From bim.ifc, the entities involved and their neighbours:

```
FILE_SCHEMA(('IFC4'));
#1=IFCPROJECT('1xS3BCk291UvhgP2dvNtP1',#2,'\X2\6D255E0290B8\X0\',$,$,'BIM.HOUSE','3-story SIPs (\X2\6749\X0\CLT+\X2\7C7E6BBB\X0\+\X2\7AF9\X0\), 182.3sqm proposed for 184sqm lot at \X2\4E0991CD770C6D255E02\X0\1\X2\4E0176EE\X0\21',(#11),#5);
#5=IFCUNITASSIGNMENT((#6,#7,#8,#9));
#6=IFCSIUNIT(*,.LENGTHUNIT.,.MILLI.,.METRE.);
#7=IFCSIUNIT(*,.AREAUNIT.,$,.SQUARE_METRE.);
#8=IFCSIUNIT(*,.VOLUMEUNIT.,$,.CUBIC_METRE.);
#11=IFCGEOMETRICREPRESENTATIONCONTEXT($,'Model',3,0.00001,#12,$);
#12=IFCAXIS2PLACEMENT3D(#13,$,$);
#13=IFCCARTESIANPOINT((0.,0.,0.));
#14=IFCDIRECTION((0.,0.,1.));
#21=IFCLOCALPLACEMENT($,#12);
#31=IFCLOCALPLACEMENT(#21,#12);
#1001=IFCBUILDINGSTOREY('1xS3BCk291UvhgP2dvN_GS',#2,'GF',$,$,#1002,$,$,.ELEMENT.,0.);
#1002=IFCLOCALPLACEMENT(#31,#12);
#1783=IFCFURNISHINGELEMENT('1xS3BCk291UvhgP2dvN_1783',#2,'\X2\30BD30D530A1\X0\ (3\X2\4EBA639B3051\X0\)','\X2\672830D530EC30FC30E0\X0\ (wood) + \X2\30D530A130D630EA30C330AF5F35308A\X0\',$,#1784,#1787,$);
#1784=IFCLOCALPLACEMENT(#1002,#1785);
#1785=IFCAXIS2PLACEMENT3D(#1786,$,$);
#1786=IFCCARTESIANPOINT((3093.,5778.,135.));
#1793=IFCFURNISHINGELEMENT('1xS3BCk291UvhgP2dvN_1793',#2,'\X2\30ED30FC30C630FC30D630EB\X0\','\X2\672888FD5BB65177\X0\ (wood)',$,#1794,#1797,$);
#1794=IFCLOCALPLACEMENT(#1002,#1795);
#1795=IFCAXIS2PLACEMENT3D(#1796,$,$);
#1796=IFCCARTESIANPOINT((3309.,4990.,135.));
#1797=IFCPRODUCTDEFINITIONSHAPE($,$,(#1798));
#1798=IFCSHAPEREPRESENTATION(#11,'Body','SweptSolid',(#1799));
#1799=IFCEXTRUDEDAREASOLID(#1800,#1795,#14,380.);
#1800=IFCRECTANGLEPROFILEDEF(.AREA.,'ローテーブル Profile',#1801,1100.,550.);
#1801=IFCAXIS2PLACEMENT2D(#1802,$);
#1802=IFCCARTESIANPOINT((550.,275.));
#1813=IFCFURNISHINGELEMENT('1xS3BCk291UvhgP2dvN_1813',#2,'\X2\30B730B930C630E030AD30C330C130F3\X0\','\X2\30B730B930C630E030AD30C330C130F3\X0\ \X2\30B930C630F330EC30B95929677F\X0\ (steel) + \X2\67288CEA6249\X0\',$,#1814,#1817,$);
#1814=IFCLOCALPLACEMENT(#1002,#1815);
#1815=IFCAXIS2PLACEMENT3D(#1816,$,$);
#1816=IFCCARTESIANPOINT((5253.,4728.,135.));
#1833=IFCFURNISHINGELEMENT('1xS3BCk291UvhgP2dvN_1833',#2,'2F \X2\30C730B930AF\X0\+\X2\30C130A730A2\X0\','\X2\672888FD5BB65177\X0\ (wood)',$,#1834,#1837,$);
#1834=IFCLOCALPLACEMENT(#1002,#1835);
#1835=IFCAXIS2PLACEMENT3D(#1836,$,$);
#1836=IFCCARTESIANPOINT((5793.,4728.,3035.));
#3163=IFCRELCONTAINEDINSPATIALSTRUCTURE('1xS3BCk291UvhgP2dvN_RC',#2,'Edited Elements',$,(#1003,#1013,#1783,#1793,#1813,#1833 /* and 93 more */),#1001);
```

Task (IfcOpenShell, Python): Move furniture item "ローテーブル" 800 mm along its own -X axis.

```python
import ifcopenshell
import ifcopenshell.api.geometry
import ifcopenshell.util.placement
import ifcopenshell.util.unit

model = ifcopenshell.open("bim.ifc")
unit_scale = ifcopenshell.util.unit.calculate_unit_scale(model)

item = model.by_guid("1xS3BCk291UvhgP2dvN_1793")
matrix = ifcopenshell.util.placement.get_local_placement(item.ObjectPlacement)
matrix[:3, 3] -= matrix[:3, 0] * 0.8 / unit_scale
ifcopenshell.api.geometry.edit_object_placement(model, product=item, matrix=matrix, is_si=False)

print(ifcopenshell.util.placement.get_local_placement(item.ObjectPlacement).round(3) + 0.0)

model.write("bim_v2.ifc")
```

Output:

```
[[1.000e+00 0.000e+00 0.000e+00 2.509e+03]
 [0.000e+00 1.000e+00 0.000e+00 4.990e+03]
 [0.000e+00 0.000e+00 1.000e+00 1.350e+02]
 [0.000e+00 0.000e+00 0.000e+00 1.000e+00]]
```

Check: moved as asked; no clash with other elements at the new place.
